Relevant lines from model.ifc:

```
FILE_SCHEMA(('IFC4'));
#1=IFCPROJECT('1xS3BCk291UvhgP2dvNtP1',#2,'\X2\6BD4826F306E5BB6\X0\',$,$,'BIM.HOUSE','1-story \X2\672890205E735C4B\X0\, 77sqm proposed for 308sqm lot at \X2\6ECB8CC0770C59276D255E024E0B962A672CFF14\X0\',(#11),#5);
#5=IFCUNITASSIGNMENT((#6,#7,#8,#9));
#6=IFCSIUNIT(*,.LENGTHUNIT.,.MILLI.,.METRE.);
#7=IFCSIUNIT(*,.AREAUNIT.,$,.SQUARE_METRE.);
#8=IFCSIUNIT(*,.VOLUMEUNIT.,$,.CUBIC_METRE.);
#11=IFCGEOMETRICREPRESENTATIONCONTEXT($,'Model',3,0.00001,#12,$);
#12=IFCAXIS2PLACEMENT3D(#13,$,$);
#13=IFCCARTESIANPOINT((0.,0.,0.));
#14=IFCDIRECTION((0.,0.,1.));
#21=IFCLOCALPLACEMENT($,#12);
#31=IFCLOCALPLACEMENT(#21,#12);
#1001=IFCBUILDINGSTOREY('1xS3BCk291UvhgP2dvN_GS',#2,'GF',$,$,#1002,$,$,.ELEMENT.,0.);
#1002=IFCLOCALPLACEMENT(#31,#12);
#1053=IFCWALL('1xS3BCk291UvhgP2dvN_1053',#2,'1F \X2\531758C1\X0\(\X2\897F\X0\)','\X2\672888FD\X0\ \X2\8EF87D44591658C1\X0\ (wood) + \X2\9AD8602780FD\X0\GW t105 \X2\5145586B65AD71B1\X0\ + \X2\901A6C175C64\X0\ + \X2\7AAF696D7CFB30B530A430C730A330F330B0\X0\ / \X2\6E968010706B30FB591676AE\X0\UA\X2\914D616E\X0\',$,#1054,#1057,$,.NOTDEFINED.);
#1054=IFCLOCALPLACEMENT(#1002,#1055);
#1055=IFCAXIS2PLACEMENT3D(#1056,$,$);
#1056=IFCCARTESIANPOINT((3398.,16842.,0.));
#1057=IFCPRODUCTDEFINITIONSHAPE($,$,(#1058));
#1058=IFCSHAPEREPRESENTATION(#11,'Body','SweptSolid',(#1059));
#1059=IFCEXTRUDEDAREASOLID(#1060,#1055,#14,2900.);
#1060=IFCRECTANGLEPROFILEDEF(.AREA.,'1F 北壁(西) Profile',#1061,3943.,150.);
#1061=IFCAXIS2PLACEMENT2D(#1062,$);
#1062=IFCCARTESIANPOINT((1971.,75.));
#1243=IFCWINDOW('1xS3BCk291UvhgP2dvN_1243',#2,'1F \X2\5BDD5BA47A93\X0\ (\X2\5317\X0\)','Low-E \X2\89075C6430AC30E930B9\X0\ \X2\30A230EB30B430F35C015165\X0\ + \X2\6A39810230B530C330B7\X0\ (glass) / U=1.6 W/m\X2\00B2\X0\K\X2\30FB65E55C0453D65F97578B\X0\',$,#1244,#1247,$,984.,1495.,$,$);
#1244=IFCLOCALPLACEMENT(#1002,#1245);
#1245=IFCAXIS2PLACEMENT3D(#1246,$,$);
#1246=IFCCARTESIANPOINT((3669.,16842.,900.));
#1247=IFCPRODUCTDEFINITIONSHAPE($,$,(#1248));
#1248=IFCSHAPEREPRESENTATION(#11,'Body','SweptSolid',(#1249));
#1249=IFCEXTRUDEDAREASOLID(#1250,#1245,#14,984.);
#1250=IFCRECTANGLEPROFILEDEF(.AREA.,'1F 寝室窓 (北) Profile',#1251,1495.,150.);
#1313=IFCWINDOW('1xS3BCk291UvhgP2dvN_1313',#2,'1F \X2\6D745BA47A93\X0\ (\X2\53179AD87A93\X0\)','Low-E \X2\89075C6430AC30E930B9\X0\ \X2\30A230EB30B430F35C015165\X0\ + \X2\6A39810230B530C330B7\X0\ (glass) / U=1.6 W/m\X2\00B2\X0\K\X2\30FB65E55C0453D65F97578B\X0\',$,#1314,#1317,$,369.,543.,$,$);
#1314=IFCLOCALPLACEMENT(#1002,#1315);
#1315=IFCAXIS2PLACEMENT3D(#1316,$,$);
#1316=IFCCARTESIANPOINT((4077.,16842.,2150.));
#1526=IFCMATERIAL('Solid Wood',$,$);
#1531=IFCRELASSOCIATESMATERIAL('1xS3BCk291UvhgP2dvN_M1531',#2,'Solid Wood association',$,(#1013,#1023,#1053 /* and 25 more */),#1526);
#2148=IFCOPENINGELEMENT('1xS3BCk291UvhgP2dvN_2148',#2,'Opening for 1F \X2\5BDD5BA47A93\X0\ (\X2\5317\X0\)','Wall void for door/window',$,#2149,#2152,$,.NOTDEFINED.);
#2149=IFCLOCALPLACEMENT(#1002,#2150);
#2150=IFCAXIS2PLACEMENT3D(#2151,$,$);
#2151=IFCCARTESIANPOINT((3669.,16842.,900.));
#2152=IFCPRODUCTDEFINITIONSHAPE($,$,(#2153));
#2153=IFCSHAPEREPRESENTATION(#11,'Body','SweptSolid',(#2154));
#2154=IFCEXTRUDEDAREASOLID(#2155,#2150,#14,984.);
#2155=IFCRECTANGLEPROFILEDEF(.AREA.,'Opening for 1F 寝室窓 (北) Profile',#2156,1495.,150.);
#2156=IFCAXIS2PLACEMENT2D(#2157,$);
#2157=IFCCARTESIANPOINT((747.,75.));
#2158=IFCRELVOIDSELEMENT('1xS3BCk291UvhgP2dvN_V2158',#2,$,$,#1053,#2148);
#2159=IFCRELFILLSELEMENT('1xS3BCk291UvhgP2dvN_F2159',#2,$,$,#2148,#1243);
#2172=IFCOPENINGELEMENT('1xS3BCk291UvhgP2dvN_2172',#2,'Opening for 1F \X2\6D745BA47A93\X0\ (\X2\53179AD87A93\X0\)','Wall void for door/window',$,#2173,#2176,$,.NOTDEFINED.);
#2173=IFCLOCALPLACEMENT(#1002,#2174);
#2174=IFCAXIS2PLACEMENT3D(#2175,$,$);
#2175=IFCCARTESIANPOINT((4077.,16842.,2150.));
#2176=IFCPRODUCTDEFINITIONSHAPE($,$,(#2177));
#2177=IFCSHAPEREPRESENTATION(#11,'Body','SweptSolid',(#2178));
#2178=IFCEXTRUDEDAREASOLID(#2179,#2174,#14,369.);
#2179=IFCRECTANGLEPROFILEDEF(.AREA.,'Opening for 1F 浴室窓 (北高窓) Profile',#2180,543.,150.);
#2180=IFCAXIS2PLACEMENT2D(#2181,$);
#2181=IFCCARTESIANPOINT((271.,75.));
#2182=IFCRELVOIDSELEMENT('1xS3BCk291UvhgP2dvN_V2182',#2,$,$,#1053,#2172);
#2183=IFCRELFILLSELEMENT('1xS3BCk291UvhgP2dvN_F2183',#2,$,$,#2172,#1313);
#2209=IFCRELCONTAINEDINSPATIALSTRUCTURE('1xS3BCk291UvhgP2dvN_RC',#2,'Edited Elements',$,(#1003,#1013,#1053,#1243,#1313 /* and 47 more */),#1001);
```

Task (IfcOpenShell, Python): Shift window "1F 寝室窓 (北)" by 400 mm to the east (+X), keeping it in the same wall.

```python
import ifcopenshell
import ifcopenshell.api.geometry
import ifcopenshell.util.placement

model = ifcopenshell.open("model.ifc")

window = model.by_guid("1xS3BCk291UvhgP2dvN_1243")
opening = window.FillsVoids[0].RelatingOpeningElement
wall = opening.VoidsElements[0].RelatingBuildingElement

wall_matrix = ifcopenshell.util.placement.get_local_placement(wall.ObjectPlacement)
shift = wall_matrix[:3, 0] * 400.0
before = ifcopenshell.util.placement.get_local_placement(window.ObjectPlacement)[:3, 3].copy()

# The window is not placed relative to its opening, so move both.
for product in (opening, window):
    matrix = ifcopenshell.util.placement.get_local_placement(product.ObjectPlacement)
    matrix[:3, 3] += shift
    ifcopenshell.api.geometry.edit_object_placement(model, product=product, matrix=matrix, is_si=False)

after = ifcopenshell.util.placement.get_local_placement(window.ObjectPlacement)[:3, 3]
print("window moved by", (after - before).round(3) + 0.0)

model.write("model-out.ifc")
```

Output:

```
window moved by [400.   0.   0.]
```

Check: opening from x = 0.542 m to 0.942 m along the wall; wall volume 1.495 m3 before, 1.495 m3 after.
